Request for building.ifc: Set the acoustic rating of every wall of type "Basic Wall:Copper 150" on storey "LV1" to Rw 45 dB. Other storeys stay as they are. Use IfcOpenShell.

First a look at what the model holds.

```python
import ifcopenshell
import ifcopenshell.util.element

model = ifcopenshell.open("building.ifc")
print(model.schema)
storey = next(s for s in model.by_type("IfcBuildingStorey") if s.Name == "LV1")
walls = [e for e in ifcopenshell.util.element.get_decomposition(storey) if e.is_a("IfcWall")]
seen = {}
for e in walls:
    element_type = ifcopenshell.util.element.get_type(e)
    key = (element_type.Name if element_type != e and element_type else None, ifcopenshell.util.element.get_pset(e, "Pset_WallCommon", "AcousticRating"))
    seen[key] = seen.get(key, 0) + 1
for (name, value), count in sorted(seen.items(), key=str):
    print(count, "x", name, "|", value)
```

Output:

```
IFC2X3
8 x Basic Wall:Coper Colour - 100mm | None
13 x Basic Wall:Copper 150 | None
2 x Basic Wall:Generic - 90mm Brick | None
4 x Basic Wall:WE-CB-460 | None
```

```python
import ifcopenshell
import ifcopenshell.api.pset
import ifcopenshell.util.element

model = ifcopenshell.open("building.ifc")

storey = next(s for s in model.by_type("IfcBuildingStorey") if s.Name == "LV1")
walls = [e for e in ifcopenshell.util.element.get_decomposition(storey) if e.is_a("IfcWall")]

count = 0
for e in walls:
    element_type = ifcopenshell.util.element.get_type(e)
    if element_type in (None, e) or element_type.Name != "Basic Wall:Copper 150":
        continue
    # add_pset returns the element's existing set when there is one.
    pset = ifcopenshell.api.pset.add_pset(model, product=e, name="Pset_WallCommon")
    ifcopenshell.api.pset.edit_pset(model, pset=pset, properties={"AcousticRating": "Rw 45 dB"})
    count += 1

print(count, "walls updated")

model.write("building_rev.ifc")
```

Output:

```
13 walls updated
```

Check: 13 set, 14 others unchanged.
